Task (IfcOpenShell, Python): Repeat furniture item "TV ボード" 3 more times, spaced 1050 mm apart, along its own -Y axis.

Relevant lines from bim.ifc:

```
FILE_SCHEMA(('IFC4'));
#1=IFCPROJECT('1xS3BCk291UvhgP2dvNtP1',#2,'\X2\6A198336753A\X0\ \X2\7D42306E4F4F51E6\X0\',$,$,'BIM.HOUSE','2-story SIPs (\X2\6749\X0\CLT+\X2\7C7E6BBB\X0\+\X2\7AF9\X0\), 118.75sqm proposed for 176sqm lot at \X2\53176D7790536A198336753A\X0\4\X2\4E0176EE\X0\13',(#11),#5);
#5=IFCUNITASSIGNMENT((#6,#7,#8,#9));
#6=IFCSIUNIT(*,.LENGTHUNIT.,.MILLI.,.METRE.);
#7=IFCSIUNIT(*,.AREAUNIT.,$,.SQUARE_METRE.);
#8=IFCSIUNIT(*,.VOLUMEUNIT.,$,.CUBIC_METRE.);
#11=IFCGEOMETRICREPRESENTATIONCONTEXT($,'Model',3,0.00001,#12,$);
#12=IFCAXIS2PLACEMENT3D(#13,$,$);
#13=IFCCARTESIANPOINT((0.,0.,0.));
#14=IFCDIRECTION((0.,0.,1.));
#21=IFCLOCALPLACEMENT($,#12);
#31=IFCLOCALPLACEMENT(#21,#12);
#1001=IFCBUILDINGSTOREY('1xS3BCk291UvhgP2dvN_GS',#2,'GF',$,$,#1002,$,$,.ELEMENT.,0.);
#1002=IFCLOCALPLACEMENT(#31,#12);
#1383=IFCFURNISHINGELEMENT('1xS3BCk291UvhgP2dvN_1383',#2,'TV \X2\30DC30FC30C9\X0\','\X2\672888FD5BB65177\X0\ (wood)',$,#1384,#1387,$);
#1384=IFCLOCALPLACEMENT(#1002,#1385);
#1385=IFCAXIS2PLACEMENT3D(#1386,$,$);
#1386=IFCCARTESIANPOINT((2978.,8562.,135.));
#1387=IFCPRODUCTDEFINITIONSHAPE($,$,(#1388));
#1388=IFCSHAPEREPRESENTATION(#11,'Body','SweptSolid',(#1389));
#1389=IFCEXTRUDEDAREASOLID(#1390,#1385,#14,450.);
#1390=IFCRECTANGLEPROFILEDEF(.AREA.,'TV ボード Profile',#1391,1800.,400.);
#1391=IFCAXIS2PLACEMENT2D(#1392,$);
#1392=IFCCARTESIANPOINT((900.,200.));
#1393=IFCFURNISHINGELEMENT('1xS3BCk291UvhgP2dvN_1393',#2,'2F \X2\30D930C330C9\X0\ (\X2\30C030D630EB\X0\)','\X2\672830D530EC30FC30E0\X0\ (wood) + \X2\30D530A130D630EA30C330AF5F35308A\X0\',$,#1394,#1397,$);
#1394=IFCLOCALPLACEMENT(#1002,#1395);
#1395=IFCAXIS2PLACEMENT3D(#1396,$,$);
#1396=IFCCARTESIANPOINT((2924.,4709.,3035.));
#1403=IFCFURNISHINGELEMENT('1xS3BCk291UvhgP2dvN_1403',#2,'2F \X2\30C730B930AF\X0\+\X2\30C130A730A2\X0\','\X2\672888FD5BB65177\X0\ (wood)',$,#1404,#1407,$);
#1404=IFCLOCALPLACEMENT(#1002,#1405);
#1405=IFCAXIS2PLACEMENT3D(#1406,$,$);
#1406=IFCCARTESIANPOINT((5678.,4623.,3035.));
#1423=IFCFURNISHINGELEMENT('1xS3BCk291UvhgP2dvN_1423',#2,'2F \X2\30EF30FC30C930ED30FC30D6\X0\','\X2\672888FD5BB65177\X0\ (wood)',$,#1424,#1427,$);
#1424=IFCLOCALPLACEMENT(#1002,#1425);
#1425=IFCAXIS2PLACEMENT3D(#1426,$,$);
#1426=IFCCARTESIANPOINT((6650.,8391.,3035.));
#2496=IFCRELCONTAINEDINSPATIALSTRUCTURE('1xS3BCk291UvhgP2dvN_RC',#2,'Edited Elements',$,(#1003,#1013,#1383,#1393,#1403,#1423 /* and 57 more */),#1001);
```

```python
import ifcopenshell
import ifcopenshell.api.geometry
import ifcopenshell.api.root
import ifcopenshell.util.element
import ifcopenshell.util.placement
import ifcopenshell.util.unit

model = ifcopenshell.open("bim.ifc")
unit_scale = ifcopenshell.util.unit.calculate_unit_scale(model)


def reuse_history(source, copy):
    """copy_class also copies each property set's owner history, people and application; keep the originals."""
    for rel in copy.IsDefinedBy:
        if rel.is_a("IfcRelDefinesByProperties") and (history := rel.RelatingPropertyDefinition.OwnerHistory):
            rel.RelatingPropertyDefinition.OwnerHistory = source.OwnerHistory
            ifcopenshell.util.element.remove_deep2(model, history)


source = model.by_id(1383)
base = ifcopenshell.util.placement.get_local_placement(source.ObjectPlacement)
step = -base[:3, 1] * 1.05 / unit_scale

for i in range(1, 4):
    copy = ifcopenshell.api.root.copy_class(model, product=source)
    copy.Representation = ifcopenshell.util.element.copy_deep(
        model, source.Representation, exclude=["IfcGeometricRepresentationContext", "IfcRepresentationMap"]
    )
    reuse_history(source, copy)
    matrix = base.copy()
    matrix[:3, 3] += i * step
    print("added at", matrix[:3, 3].round(3) + 0.0)
    ifcopenshell.api.geometry.edit_object_placement(model, product=copy, matrix=matrix, is_si=False)

model.write("bim_updated.ifc")
```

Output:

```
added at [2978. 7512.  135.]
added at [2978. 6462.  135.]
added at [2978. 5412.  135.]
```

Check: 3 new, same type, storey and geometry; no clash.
